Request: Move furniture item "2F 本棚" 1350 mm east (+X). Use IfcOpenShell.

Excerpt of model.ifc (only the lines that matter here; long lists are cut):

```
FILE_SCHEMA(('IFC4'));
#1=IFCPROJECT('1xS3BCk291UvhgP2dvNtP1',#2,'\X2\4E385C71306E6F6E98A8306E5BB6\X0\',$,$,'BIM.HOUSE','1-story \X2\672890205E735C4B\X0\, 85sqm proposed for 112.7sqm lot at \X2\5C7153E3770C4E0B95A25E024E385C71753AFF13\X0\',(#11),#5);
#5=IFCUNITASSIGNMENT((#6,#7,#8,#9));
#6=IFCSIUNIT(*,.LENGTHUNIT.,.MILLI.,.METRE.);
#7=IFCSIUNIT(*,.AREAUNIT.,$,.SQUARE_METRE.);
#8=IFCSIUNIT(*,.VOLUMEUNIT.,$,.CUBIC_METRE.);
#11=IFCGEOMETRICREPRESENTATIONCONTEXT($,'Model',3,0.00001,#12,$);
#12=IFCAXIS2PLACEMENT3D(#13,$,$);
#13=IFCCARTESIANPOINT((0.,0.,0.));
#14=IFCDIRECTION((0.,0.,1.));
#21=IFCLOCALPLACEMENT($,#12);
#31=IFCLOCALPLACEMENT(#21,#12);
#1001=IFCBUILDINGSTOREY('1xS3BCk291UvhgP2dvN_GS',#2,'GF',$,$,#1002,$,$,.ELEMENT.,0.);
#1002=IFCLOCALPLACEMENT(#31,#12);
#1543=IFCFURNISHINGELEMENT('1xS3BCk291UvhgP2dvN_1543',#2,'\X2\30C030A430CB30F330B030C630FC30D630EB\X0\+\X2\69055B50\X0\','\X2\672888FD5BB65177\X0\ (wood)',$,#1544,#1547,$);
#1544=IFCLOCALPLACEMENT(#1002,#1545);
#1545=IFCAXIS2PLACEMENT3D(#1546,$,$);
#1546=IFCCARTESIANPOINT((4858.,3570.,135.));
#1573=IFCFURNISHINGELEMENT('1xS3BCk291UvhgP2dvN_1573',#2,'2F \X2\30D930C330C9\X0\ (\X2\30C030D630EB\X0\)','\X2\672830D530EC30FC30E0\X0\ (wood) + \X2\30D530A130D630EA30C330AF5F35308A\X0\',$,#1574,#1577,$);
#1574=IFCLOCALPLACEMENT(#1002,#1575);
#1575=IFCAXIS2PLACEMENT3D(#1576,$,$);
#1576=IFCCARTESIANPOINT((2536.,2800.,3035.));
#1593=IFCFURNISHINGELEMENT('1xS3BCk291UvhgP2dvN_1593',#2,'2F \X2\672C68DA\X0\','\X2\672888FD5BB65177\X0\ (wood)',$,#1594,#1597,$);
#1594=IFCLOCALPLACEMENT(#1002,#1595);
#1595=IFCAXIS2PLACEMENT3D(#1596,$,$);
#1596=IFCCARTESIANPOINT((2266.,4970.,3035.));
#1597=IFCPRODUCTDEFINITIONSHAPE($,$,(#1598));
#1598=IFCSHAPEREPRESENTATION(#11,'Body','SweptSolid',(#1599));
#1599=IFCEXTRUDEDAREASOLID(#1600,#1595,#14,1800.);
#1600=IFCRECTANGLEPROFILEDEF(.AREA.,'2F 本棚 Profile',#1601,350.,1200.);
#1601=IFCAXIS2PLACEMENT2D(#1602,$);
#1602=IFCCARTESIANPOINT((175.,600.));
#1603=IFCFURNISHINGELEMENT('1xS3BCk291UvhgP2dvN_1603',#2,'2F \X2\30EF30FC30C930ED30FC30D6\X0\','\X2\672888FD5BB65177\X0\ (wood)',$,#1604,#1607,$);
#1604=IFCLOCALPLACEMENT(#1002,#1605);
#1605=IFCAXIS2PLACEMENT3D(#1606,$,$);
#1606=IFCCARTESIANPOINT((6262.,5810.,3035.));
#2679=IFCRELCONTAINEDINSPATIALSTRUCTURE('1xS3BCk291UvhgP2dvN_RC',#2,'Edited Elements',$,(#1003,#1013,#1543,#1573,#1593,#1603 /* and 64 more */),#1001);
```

```python
import ifcopenshell
import ifcopenshell.api.geometry
import ifcopenshell.util.placement
import ifcopenshell.util.unit

model = ifcopenshell.open("model.ifc")
unit_scale = ifcopenshell.util.unit.calculate_unit_scale(model)

item = model.by_id(1593)
matrix = ifcopenshell.util.placement.get_local_placement(item.ObjectPlacement)
matrix[0, 3] += 1.35 / unit_scale
ifcopenshell.api.geometry.edit_object_placement(model, product=item, matrix=matrix, is_si=False)

print(ifcopenshell.util.placement.get_local_placement(item.ObjectPlacement).round(3) + 0.0)

model.write("model_edited.ifc")
```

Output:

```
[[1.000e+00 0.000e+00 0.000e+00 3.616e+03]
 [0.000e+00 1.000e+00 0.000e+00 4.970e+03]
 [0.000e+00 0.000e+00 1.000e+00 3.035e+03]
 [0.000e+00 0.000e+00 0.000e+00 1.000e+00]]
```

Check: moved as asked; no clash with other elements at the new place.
